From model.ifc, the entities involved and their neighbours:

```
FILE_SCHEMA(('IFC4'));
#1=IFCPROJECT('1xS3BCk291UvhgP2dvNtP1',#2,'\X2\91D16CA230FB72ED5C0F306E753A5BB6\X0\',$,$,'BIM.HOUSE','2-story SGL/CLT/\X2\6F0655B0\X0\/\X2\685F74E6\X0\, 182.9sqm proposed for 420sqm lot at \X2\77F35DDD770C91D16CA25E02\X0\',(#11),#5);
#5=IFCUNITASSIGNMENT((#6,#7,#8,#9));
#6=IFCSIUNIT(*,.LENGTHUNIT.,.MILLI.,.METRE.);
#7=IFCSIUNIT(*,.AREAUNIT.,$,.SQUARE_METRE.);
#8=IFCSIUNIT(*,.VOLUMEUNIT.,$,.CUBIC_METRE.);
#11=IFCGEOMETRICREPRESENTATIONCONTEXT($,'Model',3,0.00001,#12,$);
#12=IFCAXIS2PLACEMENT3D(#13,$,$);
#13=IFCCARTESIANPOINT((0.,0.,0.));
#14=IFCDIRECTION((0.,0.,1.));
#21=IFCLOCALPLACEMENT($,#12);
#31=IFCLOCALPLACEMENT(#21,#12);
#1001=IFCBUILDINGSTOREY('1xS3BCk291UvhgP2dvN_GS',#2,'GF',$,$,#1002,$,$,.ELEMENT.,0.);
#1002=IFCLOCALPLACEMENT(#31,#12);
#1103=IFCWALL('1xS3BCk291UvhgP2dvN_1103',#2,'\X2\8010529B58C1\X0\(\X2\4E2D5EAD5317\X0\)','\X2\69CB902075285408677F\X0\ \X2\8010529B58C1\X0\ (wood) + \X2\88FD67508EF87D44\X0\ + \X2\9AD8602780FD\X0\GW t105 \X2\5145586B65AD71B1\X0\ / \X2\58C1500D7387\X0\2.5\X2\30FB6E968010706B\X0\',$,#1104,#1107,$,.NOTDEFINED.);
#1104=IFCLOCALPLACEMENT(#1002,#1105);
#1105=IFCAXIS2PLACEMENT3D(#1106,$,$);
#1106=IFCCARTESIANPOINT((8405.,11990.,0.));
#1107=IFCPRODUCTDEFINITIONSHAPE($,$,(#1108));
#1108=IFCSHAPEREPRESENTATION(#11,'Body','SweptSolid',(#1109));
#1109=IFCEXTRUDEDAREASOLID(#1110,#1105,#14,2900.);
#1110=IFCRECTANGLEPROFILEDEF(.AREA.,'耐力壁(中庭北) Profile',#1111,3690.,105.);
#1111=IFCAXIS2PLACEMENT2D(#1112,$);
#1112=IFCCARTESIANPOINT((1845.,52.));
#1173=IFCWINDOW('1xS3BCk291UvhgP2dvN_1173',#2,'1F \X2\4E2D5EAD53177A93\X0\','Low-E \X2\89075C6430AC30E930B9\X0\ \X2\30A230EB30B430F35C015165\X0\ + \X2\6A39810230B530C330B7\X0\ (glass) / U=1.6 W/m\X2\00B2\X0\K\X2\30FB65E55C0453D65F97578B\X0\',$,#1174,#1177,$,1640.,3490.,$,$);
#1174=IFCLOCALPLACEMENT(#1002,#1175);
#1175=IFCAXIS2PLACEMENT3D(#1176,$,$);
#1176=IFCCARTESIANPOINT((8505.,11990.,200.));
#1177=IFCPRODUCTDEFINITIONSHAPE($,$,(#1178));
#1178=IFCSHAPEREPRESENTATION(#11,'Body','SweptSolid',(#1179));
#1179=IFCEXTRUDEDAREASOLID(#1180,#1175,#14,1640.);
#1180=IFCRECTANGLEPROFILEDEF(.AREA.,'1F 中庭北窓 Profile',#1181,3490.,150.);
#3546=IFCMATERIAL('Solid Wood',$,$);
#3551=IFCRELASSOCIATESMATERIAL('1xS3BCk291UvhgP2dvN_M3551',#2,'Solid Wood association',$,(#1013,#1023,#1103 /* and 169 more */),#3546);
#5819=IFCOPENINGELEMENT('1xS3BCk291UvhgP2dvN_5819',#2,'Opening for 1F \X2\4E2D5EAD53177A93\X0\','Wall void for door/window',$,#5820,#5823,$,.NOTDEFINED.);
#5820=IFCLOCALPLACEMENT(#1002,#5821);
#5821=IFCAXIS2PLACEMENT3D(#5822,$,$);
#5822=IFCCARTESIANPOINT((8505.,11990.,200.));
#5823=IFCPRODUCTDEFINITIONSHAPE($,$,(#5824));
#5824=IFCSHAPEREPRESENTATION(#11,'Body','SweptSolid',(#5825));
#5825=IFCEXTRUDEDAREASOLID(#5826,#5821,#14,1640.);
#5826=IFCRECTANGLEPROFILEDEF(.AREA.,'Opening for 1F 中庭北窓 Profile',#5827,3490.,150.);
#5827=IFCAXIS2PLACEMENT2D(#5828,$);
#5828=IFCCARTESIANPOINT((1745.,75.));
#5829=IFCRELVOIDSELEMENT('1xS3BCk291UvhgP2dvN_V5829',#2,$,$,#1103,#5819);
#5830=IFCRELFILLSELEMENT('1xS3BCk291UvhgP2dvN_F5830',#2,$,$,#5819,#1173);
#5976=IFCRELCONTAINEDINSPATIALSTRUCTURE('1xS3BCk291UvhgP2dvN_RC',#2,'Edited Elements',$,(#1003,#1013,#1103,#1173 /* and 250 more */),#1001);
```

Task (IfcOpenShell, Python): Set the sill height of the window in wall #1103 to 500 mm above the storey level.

```python
import numpy as np
import ifcopenshell
import ifcopenshell.api.geometry
import ifcopenshell.geom
import ifcopenshell.util.element
import ifcopenshell.util.placement
import ifcopenshell.util.shape
import ifcopenshell.util.unit

model = ifcopenshell.open("model.ifc")
unit_scale = ifcopenshell.util.unit.calculate_unit_scale(model)

window = model.by_id(1173)
opening = window.FillsVoids[0].RelatingOpeningElement
storey = ifcopenshell.util.element.get_container(window, ifc_class="IfcBuildingStorey")
level = ifcopenshell.util.placement.get_local_placement(storey.ObjectPlacement)[2, 3]

# The opening's origin need not be at the sill, so measure its lowest point.
shape = ifcopenshell.geom.create_shape(ifcopenshell.geom.settings(), opening)
bottom = ifcopenshell.util.shape.get_shape_bottom_elevation(shape, shape.geometry) / unit_scale
dz = level + 500.0 - bottom

shift = np.array([0.0, 0.0, dz])
# The window is not placed relative to its opening, so move both.
for product in (opening, window):
    matrix = ifcopenshell.util.placement.get_local_placement(product.ObjectPlacement)
    matrix[:3, 3] += shift
    ifcopenshell.api.geometry.edit_object_placement(model, product=product, matrix=matrix, is_si=False)

print(f"moved by {dz * unit_scale:+.3f} m")

model.write("model_rev.ifc")
```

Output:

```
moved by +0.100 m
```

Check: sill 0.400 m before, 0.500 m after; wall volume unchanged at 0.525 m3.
